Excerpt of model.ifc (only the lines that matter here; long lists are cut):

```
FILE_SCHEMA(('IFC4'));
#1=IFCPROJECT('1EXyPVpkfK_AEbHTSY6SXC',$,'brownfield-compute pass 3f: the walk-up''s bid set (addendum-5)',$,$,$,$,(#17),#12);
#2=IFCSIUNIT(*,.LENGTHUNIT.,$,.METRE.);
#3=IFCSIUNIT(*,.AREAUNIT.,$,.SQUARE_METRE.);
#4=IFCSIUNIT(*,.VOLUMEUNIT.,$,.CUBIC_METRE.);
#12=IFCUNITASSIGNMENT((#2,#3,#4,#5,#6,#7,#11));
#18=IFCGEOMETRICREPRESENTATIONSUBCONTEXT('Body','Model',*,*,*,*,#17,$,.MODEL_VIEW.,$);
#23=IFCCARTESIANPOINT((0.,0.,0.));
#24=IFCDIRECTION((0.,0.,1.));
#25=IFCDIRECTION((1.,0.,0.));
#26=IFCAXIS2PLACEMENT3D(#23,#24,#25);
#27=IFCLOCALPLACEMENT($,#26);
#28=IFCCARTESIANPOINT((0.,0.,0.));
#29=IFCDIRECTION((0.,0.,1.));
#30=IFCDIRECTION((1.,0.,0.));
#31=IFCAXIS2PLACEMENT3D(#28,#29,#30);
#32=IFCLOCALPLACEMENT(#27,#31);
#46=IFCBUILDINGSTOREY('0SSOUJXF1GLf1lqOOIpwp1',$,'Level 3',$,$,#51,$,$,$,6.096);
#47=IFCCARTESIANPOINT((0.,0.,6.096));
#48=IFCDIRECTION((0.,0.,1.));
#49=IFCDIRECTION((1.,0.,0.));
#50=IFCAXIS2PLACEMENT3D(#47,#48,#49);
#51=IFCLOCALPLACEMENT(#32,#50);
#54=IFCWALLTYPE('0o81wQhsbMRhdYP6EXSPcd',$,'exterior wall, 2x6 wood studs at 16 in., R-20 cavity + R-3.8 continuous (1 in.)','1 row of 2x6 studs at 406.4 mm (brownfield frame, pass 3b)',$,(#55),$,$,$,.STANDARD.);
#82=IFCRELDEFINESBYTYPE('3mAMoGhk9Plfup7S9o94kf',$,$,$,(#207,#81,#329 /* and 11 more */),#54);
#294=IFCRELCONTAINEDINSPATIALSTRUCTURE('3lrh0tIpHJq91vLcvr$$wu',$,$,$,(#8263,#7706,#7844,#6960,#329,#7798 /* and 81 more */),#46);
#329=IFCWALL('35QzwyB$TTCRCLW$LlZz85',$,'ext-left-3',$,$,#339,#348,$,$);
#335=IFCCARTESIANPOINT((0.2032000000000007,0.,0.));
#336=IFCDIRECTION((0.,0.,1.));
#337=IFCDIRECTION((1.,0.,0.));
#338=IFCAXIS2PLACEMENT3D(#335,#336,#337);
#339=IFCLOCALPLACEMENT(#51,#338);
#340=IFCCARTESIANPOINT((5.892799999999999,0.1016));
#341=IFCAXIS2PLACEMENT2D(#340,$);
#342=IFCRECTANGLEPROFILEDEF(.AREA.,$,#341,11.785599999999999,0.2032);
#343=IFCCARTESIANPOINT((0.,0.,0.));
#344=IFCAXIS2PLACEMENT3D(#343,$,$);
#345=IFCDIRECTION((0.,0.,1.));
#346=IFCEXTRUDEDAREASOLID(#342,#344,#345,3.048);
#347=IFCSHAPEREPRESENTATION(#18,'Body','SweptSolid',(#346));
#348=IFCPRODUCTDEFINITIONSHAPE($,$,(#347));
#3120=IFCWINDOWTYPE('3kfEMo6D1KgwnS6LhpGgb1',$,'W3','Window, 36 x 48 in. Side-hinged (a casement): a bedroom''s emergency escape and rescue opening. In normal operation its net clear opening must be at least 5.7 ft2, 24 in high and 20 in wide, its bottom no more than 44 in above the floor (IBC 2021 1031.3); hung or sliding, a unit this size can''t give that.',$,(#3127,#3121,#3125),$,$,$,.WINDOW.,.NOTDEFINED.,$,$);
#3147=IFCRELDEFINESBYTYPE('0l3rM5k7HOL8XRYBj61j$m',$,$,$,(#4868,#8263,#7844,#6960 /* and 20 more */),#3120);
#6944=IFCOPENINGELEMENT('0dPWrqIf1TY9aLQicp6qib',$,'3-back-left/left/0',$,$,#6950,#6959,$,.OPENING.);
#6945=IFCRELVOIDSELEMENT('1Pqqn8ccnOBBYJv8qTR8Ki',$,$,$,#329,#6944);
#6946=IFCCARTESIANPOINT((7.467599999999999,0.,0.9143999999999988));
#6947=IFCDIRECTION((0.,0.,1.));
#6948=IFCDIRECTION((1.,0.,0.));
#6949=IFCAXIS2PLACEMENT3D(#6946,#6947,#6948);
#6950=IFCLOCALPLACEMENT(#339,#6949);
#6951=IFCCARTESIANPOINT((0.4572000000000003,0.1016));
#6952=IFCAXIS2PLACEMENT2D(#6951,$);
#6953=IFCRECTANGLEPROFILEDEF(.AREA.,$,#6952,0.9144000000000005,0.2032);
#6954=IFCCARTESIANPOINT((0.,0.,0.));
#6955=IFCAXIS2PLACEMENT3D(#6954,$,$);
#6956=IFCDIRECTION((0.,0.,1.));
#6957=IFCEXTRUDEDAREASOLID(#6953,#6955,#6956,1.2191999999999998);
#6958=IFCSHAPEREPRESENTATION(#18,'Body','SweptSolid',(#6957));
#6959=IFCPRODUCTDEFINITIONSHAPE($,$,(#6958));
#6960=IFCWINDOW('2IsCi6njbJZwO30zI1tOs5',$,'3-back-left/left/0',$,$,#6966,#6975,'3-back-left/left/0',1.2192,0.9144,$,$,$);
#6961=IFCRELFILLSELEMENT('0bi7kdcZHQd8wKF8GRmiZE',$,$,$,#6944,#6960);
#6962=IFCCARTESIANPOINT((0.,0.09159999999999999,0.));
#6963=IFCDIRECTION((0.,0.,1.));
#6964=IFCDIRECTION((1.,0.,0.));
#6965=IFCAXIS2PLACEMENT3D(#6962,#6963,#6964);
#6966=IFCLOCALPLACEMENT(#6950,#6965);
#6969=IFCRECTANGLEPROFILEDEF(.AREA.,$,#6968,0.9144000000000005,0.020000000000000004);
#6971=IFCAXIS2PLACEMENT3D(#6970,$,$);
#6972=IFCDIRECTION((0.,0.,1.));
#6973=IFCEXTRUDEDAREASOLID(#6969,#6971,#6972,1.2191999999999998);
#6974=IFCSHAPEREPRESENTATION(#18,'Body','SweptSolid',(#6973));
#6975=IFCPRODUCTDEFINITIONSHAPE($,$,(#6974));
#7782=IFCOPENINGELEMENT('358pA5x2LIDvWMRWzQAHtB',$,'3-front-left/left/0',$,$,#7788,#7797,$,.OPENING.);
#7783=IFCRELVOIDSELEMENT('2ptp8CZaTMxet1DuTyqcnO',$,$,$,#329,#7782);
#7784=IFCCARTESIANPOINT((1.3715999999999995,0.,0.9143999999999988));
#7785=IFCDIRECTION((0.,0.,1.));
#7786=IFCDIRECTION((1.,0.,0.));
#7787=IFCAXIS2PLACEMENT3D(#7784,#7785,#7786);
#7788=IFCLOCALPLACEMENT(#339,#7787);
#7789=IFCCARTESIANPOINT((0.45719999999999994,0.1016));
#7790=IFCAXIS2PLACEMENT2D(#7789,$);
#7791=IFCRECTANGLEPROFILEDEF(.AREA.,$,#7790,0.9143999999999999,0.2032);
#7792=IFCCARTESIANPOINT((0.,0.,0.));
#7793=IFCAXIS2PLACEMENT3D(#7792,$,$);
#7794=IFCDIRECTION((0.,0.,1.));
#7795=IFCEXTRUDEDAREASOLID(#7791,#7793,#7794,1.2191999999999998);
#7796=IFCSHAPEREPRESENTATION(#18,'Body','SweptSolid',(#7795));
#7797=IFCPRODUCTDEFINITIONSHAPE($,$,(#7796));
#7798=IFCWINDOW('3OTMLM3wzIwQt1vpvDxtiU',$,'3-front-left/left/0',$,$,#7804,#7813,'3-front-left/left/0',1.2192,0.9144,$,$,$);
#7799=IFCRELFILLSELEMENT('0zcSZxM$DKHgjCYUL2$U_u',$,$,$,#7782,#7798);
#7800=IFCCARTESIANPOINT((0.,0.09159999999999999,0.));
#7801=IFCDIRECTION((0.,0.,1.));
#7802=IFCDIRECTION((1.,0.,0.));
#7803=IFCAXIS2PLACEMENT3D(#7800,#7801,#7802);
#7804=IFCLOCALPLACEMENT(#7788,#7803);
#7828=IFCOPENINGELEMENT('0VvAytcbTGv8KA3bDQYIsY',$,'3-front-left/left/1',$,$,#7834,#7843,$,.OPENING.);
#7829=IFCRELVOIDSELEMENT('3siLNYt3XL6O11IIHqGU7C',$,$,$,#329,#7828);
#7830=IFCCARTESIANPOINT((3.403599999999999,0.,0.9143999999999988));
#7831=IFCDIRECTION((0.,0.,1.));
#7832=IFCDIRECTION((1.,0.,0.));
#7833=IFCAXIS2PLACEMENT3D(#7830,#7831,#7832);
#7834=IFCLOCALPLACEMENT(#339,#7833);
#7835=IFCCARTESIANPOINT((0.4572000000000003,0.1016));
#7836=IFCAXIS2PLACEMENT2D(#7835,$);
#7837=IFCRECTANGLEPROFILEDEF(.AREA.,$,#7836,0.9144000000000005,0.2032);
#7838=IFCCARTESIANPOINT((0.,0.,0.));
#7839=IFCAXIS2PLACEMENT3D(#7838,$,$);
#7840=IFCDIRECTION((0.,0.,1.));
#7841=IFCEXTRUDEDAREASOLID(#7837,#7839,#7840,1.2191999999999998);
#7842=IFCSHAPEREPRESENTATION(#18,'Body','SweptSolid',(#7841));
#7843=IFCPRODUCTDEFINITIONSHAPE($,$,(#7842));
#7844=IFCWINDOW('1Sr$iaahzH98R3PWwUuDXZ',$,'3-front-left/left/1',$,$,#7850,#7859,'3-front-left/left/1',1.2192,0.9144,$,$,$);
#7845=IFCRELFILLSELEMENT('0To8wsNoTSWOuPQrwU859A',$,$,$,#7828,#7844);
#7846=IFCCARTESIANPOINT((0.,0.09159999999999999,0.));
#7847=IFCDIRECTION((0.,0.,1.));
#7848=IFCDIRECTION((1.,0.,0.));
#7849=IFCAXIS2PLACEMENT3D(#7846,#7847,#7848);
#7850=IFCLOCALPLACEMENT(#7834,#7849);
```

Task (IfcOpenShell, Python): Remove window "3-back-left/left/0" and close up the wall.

```python
import ifcopenshell
import ifcopenshell.api.feature
import ifcopenshell.api.root
import ifcopenshell.geom
import ifcopenshell.util.shape

model = ifcopenshell.open("model.ifc")
settings = ifcopenshell.geom.settings()


def volume(element):
    """Net volume in cubic metres, openings subtracted."""
    shape = ifcopenshell.geom.create_shape(settings, element)
    return ifcopenshell.util.shape.get_volume(shape.geometry)


window = model.by_guid("2IsCi6njbJZwO30zI1tOs5")
opening = window.FillsVoids[0].RelatingOpeningElement
wall = opening.VoidsElements[0].RelatingBuildingElement
before = volume(wall)

ifcopenshell.api.root.remove_product(model, product=window)
ifcopenshell.api.feature.remove_feature(model, feature=opening)

after = volume(wall)

print(f"wall volume {before:.3f} -> {after:.3f} m3")

model.write("model_updated.ifc")
```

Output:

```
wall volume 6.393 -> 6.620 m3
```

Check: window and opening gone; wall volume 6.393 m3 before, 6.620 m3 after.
